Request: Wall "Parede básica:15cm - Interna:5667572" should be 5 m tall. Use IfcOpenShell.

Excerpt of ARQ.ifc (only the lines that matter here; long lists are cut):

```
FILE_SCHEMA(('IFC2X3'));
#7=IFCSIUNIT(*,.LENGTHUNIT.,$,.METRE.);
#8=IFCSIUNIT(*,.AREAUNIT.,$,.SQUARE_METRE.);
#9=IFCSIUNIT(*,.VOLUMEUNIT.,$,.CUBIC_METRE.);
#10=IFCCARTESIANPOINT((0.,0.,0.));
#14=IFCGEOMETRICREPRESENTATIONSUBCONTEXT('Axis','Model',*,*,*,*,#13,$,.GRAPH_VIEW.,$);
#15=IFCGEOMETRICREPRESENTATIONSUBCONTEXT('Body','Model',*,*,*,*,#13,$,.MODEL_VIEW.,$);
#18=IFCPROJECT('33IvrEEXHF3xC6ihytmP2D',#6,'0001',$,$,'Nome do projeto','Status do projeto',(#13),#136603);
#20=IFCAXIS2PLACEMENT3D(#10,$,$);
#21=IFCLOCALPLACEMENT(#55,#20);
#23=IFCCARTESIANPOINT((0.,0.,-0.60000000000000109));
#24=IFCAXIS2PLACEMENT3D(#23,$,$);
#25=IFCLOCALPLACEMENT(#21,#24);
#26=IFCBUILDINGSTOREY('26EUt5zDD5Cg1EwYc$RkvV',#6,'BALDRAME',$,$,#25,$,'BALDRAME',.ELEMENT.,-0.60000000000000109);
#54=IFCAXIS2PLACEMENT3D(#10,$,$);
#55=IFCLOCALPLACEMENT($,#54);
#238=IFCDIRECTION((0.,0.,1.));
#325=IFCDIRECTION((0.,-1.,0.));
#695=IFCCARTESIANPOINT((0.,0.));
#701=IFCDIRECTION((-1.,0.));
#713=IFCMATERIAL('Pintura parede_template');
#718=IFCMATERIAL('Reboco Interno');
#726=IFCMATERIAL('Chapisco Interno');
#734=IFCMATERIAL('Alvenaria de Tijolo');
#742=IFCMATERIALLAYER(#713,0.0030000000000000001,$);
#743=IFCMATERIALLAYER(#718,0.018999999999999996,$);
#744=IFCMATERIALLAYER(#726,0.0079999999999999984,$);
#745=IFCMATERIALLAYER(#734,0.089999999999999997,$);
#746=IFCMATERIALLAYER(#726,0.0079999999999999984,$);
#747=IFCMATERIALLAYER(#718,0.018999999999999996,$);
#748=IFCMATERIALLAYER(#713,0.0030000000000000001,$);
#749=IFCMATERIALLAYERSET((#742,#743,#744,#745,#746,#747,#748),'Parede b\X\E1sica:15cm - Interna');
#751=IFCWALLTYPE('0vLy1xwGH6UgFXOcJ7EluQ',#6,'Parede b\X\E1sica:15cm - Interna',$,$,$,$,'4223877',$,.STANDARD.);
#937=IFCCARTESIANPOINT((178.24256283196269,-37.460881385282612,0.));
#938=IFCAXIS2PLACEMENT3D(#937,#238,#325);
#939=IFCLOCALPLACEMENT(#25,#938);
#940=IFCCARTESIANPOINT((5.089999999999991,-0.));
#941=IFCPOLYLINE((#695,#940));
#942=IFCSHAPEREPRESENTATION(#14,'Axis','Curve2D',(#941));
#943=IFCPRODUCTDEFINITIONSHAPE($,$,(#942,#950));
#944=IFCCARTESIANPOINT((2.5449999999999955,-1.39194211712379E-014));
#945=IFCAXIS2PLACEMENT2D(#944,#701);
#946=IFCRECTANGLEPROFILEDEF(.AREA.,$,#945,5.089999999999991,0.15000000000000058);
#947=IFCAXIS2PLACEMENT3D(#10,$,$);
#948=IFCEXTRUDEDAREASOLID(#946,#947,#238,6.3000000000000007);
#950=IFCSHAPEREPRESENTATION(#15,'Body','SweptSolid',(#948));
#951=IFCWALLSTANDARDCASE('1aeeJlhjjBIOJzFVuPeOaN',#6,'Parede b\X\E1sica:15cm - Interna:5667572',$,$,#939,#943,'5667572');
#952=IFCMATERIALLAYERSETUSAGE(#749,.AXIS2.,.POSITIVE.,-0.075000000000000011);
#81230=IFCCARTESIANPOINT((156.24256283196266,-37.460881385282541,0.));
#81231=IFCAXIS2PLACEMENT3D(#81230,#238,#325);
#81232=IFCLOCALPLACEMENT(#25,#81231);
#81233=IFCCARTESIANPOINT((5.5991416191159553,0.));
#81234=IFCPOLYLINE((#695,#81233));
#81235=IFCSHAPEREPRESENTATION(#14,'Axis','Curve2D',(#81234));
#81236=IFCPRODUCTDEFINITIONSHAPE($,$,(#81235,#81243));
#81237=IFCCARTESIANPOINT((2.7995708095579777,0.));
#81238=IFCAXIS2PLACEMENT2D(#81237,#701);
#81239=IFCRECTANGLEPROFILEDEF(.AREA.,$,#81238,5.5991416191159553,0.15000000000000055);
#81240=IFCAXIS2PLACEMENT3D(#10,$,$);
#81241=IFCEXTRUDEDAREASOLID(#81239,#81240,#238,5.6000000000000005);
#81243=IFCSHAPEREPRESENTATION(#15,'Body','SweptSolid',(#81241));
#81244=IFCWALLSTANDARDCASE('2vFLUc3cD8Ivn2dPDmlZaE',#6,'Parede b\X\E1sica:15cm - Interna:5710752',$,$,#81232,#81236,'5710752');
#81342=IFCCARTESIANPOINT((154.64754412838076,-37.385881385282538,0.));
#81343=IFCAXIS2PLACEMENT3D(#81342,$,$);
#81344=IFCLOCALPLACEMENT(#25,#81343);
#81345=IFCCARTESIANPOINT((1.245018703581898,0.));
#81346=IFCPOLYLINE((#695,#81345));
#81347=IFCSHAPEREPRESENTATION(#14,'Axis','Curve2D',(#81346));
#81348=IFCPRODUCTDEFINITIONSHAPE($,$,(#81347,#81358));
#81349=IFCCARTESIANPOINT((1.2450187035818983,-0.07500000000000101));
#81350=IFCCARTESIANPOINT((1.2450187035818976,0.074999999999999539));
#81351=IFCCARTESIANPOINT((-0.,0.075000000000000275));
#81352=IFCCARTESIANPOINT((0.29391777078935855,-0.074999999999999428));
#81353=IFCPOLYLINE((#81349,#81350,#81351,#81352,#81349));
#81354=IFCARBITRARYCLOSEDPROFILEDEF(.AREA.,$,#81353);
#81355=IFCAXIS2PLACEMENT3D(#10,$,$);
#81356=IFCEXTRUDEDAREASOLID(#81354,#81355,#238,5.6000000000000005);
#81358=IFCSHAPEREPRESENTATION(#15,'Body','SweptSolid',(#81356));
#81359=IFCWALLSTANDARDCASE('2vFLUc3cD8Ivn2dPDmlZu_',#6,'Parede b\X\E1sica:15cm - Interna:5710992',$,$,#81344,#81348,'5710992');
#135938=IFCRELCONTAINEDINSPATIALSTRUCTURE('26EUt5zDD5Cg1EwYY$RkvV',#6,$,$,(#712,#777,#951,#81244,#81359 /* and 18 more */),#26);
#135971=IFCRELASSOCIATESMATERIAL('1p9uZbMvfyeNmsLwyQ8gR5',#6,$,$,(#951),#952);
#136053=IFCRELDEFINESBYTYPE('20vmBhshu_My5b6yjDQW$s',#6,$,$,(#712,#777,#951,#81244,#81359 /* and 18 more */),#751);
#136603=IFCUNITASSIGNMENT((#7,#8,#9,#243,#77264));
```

```python
import ifcopenshell
import ifcopenshell.geom
import ifcopenshell.util.representation
import ifcopenshell.util.shape
import ifcopenshell.util.unit

model = ifcopenshell.open("ARQ.ifc")
unit_scale = ifcopenshell.util.unit.calculate_unit_scale(model)
settings = ifcopenshell.geom.settings()


def volume(element):
    """Net volume in cubic metres, openings subtracted."""
    shape = ifcopenshell.geom.create_shape(settings, element)
    return ifcopenshell.util.shape.get_volume(shape.geometry)


wall = model.by_guid("1aeeJlhjjBIOJzFVuPeOaN")
before = volume(wall)

body = ifcopenshell.util.representation.get_representation(wall, "Model", "Body")
solid = body.Items[0]
old_height = solid.Depth
solid.Depth = 5 / unit_scale
after = volume(wall)

print(f"height {old_height:g} -> {solid.Depth:g}, volume {before:.3f} -> {after:.3f} m3")

model.write("ARQ_v2.ifc")
```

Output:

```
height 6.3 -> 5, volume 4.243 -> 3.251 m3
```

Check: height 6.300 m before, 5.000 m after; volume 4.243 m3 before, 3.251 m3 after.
